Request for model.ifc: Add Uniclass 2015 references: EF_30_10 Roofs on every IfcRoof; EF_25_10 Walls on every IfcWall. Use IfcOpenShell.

First a look at what the model holds.

```python
import ifcopenshell

model = ifcopenshell.open("model.ifc")
print(model.schema)
print("classifications:", [c.Name for c in model.by_type("IfcClassification")])
for ifc_class in ("IfcDoor", "IfcRoof", "IfcStair", "IfcWall", "IfcWindow"):
    print(ifc_class, len(model.by_type(ifc_class)))
```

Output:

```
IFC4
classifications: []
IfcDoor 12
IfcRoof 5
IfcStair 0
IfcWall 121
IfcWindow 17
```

```python
import ifcopenshell
import ifcopenshell.api.classification

model = ifcopenshell.open("model.ifc")

system = ifcopenshell.api.classification.add_classification(model, classification="Uniclass 2015")

codes = {
    "IfcRoof": ("EF_30_10", "Roofs"),
    "IfcWall": ("EF_25_10", "Walls"),
}
for ifc_class, (code, name) in codes.items():
    products = model.by_type(ifc_class)
    ifcopenshell.api.classification.add_reference(
        model, products=products, classification=system, identification=code, name=name
    )
    print(code, len(products))

model.write("model_edited.ifc")
```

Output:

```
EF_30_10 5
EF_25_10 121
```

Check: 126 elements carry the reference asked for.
